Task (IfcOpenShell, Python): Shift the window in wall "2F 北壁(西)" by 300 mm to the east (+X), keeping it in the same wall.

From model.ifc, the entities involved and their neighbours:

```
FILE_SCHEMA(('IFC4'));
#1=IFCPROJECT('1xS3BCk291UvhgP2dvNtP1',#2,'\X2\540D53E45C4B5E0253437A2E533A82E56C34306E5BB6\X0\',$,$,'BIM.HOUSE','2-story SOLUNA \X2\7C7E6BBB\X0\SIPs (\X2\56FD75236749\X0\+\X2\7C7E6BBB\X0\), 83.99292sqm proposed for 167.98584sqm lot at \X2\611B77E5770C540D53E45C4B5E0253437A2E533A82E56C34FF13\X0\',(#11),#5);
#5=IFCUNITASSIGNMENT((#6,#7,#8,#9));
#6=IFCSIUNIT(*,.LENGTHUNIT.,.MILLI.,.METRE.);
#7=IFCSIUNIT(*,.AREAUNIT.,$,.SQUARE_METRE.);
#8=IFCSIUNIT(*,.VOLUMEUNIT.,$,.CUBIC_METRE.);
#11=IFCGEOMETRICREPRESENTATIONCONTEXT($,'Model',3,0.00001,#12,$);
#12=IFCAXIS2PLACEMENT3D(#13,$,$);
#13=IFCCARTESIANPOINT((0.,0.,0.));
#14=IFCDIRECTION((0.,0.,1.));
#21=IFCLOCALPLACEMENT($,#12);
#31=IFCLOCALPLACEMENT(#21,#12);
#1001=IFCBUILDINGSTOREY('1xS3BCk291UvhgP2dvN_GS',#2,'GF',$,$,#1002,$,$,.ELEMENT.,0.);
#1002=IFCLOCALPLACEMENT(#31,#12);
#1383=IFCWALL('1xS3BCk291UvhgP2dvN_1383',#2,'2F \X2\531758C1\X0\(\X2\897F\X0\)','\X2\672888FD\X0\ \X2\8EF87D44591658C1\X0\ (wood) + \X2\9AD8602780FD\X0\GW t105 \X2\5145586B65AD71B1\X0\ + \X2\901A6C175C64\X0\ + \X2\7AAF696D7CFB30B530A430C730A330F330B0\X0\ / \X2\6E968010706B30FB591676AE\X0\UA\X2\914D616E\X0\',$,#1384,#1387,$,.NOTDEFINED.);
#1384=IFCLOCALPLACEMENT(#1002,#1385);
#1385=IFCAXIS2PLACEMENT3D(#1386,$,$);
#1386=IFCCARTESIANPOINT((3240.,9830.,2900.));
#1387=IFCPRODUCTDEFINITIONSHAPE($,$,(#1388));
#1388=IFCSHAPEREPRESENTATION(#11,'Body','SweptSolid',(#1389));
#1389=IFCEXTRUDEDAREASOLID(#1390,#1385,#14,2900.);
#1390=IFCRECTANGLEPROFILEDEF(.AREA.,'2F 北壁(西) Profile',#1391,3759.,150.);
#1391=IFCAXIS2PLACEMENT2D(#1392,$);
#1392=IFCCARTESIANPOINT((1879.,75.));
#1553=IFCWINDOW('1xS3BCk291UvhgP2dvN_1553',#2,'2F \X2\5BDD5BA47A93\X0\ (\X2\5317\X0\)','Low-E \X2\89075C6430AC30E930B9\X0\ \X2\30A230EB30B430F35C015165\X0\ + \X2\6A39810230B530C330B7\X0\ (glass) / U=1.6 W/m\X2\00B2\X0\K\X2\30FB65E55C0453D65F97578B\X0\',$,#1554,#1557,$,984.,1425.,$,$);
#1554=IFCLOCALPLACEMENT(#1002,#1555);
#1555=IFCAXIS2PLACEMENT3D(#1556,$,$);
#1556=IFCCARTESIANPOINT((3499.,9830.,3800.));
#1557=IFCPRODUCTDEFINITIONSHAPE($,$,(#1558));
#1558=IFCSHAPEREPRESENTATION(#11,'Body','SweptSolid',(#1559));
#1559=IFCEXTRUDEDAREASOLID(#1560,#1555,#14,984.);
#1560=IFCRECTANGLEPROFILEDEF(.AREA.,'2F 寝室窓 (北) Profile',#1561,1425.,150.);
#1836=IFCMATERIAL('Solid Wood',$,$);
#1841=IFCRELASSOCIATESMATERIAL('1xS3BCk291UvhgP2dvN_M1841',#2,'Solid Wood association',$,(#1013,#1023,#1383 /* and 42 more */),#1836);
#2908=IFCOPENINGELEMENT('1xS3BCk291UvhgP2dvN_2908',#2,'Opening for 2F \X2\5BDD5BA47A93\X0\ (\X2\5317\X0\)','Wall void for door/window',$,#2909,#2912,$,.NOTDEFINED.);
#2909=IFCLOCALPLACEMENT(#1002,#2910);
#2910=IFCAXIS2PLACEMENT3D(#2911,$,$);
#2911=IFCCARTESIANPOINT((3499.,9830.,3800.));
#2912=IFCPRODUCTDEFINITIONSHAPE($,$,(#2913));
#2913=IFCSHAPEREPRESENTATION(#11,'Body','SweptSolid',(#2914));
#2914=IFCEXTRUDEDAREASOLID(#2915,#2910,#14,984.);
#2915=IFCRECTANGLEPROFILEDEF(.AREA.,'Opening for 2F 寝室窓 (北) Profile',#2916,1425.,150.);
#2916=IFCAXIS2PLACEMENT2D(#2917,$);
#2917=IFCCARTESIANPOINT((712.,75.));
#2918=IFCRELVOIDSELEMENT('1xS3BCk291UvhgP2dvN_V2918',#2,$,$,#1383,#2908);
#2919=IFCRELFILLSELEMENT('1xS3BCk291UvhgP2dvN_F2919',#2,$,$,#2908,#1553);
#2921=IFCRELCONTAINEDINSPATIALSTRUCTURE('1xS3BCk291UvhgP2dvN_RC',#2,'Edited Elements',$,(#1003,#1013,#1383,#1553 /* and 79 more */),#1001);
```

```python
import ifcopenshell
import ifcopenshell.api.geometry
import ifcopenshell.util.placement
import ifcopenshell.util.unit

model = ifcopenshell.open("model.ifc")
unit_scale = ifcopenshell.util.unit.calculate_unit_scale(model)

window = model.by_id(1553)
opening = window.FillsVoids[0].RelatingOpeningElement
wall = opening.VoidsElements[0].RelatingBuildingElement

wall_matrix = ifcopenshell.util.placement.get_local_placement(wall.ObjectPlacement)
shift = wall_matrix[:3, 0] * 0.3 / unit_scale
before = ifcopenshell.util.placement.get_local_placement(window.ObjectPlacement)[:3, 3].copy()

# The window is not placed relative to its opening, so move both.
for product in (opening, window):
    matrix = ifcopenshell.util.placement.get_local_placement(product.ObjectPlacement)
    matrix[:3, 3] += shift
    ifcopenshell.api.geometry.edit_object_placement(model, product=product, matrix=matrix, is_si=False)

after = ifcopenshell.util.placement.get_local_placement(window.ObjectPlacement)[:3, 3]
print("window moved by", (after - before).round(3) + 0.0)

model.write("model-out.ifc")
```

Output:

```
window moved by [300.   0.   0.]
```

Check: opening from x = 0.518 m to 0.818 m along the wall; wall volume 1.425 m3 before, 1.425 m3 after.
